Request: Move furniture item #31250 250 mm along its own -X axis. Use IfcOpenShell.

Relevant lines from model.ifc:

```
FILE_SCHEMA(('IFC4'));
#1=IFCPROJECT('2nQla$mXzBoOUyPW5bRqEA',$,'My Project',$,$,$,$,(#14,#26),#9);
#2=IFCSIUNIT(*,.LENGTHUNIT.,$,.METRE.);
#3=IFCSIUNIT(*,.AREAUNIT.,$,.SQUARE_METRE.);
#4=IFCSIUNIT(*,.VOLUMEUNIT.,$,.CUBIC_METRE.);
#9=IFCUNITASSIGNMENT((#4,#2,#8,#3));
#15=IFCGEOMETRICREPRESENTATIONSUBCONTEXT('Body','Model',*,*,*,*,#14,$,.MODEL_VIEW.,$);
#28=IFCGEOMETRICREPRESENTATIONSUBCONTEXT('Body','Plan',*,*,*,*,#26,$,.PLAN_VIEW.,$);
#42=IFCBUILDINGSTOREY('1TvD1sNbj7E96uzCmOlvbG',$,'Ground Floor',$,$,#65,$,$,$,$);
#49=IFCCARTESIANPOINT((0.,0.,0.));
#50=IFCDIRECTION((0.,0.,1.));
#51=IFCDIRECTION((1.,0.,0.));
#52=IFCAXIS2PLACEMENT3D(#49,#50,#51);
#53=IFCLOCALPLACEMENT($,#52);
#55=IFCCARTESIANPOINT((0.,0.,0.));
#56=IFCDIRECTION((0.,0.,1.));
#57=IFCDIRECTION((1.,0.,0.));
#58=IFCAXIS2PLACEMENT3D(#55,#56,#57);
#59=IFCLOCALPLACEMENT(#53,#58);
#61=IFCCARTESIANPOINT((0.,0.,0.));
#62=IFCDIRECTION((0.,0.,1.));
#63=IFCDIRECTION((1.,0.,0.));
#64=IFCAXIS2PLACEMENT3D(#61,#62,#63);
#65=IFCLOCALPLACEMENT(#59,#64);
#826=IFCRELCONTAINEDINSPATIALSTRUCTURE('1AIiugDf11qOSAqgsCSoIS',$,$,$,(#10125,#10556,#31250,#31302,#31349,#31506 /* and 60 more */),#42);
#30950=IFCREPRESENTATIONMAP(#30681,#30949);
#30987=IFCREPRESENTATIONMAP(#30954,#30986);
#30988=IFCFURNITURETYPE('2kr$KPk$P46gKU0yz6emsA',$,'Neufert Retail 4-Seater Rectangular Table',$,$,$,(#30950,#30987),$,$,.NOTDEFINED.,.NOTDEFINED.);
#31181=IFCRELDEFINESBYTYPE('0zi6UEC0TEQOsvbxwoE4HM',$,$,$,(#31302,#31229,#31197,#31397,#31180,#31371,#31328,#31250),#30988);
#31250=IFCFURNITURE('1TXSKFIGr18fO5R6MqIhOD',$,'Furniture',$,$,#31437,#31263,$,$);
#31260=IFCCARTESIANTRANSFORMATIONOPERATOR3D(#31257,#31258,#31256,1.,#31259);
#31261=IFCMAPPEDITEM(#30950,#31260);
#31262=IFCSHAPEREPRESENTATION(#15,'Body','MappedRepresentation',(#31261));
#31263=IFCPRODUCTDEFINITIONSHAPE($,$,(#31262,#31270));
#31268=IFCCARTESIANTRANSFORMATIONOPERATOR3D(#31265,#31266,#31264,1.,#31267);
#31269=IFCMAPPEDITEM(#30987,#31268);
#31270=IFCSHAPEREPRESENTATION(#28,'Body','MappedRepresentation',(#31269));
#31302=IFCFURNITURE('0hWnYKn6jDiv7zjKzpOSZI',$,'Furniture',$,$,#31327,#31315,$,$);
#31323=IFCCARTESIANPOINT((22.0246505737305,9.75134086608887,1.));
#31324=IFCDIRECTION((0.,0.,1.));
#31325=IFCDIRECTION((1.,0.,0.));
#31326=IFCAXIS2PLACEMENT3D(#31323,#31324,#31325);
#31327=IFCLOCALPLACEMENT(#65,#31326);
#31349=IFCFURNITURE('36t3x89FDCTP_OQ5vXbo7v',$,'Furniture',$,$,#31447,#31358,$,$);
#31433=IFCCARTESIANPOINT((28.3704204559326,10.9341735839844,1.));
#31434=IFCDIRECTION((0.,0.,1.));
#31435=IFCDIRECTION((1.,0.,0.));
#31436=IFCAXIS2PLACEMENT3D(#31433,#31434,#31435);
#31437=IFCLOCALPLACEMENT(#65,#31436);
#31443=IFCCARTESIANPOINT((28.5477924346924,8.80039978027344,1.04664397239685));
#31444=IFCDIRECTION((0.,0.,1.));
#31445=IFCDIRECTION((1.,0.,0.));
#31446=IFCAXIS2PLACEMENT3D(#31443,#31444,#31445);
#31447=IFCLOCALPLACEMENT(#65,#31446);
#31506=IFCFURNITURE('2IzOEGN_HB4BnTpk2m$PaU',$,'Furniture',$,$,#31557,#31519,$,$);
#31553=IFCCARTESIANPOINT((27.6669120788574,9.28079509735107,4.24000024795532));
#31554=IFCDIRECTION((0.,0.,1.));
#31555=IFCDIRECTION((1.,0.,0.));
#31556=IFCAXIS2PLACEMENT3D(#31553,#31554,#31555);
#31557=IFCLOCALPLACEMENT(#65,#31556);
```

```python
import ifcopenshell
import ifcopenshell.api.geometry
import ifcopenshell.util.placement
import ifcopenshell.util.unit

model = ifcopenshell.open("model.ifc")
unit_scale = ifcopenshell.util.unit.calculate_unit_scale(model)

item = model.by_guid("1TXSKFIGr18fO5R6MqIhOD")
matrix = ifcopenshell.util.placement.get_local_placement(item.ObjectPlacement)
matrix[:3, 3] -= matrix[:3, 0] * 0.25 / unit_scale
ifcopenshell.api.geometry.edit_object_placement(model, product=item, matrix=matrix, is_si=False)

print(ifcopenshell.util.placement.get_local_placement(item.ObjectPlacement).round(3) + 0.0)

model.write("model_edited.ifc")
```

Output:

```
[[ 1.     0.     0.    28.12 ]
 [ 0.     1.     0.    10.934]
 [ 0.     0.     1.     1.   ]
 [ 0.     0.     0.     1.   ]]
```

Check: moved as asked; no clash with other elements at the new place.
